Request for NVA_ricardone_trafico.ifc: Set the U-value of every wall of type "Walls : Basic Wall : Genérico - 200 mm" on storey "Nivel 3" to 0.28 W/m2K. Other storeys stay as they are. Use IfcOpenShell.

First a look at what the model holds.

```python
import ifcopenshell
import ifcopenshell.util.element

model = ifcopenshell.open("NVA_ricardone_trafico.ifc")
print(model.schema)
storey = next(s for s in model.by_type("IfcBuildingStorey") if s.Name == "Nivel 3")
walls = [e for e in ifcopenshell.util.element.get_decomposition(storey) if e.is_a("IfcWall")]
seen = {}
for e in walls:
    element_type = ifcopenshell.util.element.get_type(e)
    key = (element_type.Name if element_type != e and element_type else None, ifcopenshell.util.element.get_pset(e, "Pset_WallCommon", "ThermalTransmittance"))
    seen[key] = seen.get(key, 0) + 1
for (name, value), count in sorted(seen.items(), key=str):
    print(count, "x", name, "|", value)
```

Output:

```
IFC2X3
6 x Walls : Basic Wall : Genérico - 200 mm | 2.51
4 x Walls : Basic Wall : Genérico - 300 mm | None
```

```python
import ifcopenshell
import ifcopenshell.api.pset
import ifcopenshell.util.element

model = ifcopenshell.open("NVA_ricardone_trafico.ifc")

storey = next(s for s in model.by_type("IfcBuildingStorey") if s.Name == "Nivel 3")
walls = [e for e in ifcopenshell.util.element.get_decomposition(storey) if e.is_a("IfcWall")]

count = 0
for e in walls:
    element_type = ifcopenshell.util.element.get_type(e)
    if element_type in (None, e) or element_type.Name != "Walls : Basic Wall : Genérico - 200 mm":
        continue
    # add_pset returns the element's existing set when there is one.
    pset = ifcopenshell.api.pset.add_pset(model, product=e, name="Pset_WallCommon")
    ifcopenshell.api.pset.edit_pset(model, pset=pset, properties={"ThermalTransmittance": 0.28})
    count += 1

print(count, "walls updated")

model.write("NVA_ricardone_trafico_rev.ifc")
```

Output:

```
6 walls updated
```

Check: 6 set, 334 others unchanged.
